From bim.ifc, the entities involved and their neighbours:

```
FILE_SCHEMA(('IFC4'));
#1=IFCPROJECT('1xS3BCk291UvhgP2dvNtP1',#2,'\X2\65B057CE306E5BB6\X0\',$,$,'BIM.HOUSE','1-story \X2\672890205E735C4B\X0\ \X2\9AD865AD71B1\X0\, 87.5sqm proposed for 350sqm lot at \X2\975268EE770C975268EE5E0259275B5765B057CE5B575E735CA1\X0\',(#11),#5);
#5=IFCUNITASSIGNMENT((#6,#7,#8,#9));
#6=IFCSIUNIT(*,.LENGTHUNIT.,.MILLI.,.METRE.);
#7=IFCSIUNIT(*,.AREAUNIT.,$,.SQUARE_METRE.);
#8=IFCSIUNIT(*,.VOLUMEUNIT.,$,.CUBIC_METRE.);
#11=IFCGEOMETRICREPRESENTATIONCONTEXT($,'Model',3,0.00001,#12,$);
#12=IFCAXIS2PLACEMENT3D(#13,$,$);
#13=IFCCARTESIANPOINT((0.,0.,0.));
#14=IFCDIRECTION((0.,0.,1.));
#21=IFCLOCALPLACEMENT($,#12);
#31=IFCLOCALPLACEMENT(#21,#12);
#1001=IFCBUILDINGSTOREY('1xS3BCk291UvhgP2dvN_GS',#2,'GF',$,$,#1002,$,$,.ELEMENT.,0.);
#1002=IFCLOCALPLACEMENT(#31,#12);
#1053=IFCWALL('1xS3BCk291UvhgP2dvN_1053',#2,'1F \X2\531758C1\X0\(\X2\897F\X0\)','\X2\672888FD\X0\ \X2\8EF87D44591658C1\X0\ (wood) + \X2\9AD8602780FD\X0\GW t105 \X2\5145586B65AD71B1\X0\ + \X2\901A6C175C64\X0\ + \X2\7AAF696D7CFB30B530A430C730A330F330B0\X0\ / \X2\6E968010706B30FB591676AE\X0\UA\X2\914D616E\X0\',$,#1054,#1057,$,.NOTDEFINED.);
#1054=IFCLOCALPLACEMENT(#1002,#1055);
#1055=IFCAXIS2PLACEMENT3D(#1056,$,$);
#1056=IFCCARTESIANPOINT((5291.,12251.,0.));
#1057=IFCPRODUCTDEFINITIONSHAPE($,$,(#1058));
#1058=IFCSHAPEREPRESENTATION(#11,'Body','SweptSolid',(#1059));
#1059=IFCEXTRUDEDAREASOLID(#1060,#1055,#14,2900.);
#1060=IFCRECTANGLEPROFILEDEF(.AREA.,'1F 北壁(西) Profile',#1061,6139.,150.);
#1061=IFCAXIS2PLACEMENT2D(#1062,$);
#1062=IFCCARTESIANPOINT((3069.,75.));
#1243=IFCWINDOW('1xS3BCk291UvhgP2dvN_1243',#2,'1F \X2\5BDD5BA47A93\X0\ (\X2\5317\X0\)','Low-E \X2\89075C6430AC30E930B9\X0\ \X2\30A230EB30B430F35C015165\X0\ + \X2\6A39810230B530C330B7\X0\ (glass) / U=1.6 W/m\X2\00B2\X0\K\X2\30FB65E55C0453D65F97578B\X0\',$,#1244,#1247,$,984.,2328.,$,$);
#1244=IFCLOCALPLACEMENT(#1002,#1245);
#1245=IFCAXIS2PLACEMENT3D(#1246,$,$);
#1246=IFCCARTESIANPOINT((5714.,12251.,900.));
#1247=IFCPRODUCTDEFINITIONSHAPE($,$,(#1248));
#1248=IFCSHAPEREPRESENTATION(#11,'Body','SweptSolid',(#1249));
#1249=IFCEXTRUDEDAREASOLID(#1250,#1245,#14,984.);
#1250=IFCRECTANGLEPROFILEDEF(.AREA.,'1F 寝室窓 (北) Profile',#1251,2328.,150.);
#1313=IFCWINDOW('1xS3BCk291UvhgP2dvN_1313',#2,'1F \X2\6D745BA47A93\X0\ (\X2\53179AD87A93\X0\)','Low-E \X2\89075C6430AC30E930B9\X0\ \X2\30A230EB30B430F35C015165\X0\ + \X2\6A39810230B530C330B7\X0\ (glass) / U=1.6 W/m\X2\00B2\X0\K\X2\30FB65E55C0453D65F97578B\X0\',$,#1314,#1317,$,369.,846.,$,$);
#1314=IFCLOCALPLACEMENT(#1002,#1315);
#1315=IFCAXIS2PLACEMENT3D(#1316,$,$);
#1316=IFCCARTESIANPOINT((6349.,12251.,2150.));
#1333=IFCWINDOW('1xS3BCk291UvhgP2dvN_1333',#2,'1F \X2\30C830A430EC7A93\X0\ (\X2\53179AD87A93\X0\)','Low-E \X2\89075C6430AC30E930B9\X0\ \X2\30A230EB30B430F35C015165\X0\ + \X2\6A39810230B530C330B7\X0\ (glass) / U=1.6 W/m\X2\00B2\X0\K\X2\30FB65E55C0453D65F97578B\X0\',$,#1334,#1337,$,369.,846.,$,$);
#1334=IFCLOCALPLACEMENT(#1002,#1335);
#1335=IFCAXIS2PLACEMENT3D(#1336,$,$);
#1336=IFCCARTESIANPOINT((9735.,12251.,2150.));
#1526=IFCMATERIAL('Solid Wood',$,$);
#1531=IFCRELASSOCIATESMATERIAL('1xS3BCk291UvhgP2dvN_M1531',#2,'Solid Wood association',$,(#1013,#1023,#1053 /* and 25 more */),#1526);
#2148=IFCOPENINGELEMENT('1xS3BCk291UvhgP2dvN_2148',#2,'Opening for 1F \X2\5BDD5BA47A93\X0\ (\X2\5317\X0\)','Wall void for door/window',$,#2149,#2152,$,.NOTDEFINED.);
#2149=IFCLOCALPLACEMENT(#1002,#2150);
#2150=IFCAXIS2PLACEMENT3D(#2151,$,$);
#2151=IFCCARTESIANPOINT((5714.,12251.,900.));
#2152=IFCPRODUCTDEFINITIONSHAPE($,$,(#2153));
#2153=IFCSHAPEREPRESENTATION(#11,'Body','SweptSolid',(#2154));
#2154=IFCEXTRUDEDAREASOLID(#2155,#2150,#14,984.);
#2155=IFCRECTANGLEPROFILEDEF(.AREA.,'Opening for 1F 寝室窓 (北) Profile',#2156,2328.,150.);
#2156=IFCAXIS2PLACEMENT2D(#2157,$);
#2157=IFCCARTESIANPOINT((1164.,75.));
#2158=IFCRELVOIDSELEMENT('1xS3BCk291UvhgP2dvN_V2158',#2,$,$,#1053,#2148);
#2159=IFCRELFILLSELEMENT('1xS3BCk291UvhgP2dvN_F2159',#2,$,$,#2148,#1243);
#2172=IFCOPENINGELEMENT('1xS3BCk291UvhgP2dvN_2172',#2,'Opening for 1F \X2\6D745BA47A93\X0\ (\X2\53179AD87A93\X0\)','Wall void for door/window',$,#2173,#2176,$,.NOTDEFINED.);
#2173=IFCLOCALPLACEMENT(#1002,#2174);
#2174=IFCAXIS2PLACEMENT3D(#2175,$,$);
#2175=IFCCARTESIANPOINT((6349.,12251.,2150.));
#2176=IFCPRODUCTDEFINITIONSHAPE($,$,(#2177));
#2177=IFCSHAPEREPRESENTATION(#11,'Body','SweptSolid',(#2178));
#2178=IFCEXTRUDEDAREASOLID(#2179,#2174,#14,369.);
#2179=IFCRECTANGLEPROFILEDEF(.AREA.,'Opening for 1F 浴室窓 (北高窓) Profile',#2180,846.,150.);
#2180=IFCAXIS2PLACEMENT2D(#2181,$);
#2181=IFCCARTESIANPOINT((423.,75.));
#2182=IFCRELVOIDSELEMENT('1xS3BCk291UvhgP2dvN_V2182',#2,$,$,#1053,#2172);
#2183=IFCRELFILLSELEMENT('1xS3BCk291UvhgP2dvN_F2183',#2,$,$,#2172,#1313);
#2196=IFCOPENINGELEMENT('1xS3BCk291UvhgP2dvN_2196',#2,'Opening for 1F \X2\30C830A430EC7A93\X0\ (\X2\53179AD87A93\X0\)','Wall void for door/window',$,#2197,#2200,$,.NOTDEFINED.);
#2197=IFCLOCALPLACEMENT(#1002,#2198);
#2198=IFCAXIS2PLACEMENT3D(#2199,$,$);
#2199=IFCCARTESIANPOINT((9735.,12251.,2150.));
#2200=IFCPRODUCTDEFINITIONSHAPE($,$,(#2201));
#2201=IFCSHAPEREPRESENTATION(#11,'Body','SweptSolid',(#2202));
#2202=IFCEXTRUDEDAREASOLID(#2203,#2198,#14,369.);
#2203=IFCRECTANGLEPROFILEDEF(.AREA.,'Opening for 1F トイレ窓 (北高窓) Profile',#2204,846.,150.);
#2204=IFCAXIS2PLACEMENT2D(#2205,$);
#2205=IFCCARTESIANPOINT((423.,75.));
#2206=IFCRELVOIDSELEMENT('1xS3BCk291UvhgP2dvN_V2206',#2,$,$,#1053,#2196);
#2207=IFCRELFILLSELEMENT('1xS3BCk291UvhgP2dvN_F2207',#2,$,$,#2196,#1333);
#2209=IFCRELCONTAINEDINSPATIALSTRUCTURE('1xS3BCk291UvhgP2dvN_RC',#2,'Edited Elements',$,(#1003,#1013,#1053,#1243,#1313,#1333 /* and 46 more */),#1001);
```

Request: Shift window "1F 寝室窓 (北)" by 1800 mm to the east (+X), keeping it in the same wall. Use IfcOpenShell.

```python
import ifcopenshell
import ifcopenshell.api.geometry
import ifcopenshell.util.placement
import ifcopenshell.util.unit

model = ifcopenshell.open("bim.ifc")
unit_scale = ifcopenshell.util.unit.calculate_unit_scale(model)

window = model.by_guid("1xS3BCk291UvhgP2dvN_1243")
opening = window.FillsVoids[0].RelatingOpeningElement
wall = opening.VoidsElements[0].RelatingBuildingElement

wall_matrix = ifcopenshell.util.placement.get_local_placement(wall.ObjectPlacement)
shift = wall_matrix[:3, 0] * 1.8 / unit_scale
before = ifcopenshell.util.placement.get_local_placement(window.ObjectPlacement)[:3, 3].copy()

# The window is not placed relative to its opening, so move both.
for product in (opening, window):
    matrix = ifcopenshell.util.placement.get_local_placement(product.ObjectPlacement)
    matrix[:3, 3] += shift
    ifcopenshell.api.geometry.edit_object_placement(model, product=product, matrix=matrix, is_si=False)

after = ifcopenshell.util.placement.get_local_placement(window.ObjectPlacement)[:3, 3]
print("window moved by", (after - before).round(3) + 0.0)

model.write("bim_updated.ifc")
```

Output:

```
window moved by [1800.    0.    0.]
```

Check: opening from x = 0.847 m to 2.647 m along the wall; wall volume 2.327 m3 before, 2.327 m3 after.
